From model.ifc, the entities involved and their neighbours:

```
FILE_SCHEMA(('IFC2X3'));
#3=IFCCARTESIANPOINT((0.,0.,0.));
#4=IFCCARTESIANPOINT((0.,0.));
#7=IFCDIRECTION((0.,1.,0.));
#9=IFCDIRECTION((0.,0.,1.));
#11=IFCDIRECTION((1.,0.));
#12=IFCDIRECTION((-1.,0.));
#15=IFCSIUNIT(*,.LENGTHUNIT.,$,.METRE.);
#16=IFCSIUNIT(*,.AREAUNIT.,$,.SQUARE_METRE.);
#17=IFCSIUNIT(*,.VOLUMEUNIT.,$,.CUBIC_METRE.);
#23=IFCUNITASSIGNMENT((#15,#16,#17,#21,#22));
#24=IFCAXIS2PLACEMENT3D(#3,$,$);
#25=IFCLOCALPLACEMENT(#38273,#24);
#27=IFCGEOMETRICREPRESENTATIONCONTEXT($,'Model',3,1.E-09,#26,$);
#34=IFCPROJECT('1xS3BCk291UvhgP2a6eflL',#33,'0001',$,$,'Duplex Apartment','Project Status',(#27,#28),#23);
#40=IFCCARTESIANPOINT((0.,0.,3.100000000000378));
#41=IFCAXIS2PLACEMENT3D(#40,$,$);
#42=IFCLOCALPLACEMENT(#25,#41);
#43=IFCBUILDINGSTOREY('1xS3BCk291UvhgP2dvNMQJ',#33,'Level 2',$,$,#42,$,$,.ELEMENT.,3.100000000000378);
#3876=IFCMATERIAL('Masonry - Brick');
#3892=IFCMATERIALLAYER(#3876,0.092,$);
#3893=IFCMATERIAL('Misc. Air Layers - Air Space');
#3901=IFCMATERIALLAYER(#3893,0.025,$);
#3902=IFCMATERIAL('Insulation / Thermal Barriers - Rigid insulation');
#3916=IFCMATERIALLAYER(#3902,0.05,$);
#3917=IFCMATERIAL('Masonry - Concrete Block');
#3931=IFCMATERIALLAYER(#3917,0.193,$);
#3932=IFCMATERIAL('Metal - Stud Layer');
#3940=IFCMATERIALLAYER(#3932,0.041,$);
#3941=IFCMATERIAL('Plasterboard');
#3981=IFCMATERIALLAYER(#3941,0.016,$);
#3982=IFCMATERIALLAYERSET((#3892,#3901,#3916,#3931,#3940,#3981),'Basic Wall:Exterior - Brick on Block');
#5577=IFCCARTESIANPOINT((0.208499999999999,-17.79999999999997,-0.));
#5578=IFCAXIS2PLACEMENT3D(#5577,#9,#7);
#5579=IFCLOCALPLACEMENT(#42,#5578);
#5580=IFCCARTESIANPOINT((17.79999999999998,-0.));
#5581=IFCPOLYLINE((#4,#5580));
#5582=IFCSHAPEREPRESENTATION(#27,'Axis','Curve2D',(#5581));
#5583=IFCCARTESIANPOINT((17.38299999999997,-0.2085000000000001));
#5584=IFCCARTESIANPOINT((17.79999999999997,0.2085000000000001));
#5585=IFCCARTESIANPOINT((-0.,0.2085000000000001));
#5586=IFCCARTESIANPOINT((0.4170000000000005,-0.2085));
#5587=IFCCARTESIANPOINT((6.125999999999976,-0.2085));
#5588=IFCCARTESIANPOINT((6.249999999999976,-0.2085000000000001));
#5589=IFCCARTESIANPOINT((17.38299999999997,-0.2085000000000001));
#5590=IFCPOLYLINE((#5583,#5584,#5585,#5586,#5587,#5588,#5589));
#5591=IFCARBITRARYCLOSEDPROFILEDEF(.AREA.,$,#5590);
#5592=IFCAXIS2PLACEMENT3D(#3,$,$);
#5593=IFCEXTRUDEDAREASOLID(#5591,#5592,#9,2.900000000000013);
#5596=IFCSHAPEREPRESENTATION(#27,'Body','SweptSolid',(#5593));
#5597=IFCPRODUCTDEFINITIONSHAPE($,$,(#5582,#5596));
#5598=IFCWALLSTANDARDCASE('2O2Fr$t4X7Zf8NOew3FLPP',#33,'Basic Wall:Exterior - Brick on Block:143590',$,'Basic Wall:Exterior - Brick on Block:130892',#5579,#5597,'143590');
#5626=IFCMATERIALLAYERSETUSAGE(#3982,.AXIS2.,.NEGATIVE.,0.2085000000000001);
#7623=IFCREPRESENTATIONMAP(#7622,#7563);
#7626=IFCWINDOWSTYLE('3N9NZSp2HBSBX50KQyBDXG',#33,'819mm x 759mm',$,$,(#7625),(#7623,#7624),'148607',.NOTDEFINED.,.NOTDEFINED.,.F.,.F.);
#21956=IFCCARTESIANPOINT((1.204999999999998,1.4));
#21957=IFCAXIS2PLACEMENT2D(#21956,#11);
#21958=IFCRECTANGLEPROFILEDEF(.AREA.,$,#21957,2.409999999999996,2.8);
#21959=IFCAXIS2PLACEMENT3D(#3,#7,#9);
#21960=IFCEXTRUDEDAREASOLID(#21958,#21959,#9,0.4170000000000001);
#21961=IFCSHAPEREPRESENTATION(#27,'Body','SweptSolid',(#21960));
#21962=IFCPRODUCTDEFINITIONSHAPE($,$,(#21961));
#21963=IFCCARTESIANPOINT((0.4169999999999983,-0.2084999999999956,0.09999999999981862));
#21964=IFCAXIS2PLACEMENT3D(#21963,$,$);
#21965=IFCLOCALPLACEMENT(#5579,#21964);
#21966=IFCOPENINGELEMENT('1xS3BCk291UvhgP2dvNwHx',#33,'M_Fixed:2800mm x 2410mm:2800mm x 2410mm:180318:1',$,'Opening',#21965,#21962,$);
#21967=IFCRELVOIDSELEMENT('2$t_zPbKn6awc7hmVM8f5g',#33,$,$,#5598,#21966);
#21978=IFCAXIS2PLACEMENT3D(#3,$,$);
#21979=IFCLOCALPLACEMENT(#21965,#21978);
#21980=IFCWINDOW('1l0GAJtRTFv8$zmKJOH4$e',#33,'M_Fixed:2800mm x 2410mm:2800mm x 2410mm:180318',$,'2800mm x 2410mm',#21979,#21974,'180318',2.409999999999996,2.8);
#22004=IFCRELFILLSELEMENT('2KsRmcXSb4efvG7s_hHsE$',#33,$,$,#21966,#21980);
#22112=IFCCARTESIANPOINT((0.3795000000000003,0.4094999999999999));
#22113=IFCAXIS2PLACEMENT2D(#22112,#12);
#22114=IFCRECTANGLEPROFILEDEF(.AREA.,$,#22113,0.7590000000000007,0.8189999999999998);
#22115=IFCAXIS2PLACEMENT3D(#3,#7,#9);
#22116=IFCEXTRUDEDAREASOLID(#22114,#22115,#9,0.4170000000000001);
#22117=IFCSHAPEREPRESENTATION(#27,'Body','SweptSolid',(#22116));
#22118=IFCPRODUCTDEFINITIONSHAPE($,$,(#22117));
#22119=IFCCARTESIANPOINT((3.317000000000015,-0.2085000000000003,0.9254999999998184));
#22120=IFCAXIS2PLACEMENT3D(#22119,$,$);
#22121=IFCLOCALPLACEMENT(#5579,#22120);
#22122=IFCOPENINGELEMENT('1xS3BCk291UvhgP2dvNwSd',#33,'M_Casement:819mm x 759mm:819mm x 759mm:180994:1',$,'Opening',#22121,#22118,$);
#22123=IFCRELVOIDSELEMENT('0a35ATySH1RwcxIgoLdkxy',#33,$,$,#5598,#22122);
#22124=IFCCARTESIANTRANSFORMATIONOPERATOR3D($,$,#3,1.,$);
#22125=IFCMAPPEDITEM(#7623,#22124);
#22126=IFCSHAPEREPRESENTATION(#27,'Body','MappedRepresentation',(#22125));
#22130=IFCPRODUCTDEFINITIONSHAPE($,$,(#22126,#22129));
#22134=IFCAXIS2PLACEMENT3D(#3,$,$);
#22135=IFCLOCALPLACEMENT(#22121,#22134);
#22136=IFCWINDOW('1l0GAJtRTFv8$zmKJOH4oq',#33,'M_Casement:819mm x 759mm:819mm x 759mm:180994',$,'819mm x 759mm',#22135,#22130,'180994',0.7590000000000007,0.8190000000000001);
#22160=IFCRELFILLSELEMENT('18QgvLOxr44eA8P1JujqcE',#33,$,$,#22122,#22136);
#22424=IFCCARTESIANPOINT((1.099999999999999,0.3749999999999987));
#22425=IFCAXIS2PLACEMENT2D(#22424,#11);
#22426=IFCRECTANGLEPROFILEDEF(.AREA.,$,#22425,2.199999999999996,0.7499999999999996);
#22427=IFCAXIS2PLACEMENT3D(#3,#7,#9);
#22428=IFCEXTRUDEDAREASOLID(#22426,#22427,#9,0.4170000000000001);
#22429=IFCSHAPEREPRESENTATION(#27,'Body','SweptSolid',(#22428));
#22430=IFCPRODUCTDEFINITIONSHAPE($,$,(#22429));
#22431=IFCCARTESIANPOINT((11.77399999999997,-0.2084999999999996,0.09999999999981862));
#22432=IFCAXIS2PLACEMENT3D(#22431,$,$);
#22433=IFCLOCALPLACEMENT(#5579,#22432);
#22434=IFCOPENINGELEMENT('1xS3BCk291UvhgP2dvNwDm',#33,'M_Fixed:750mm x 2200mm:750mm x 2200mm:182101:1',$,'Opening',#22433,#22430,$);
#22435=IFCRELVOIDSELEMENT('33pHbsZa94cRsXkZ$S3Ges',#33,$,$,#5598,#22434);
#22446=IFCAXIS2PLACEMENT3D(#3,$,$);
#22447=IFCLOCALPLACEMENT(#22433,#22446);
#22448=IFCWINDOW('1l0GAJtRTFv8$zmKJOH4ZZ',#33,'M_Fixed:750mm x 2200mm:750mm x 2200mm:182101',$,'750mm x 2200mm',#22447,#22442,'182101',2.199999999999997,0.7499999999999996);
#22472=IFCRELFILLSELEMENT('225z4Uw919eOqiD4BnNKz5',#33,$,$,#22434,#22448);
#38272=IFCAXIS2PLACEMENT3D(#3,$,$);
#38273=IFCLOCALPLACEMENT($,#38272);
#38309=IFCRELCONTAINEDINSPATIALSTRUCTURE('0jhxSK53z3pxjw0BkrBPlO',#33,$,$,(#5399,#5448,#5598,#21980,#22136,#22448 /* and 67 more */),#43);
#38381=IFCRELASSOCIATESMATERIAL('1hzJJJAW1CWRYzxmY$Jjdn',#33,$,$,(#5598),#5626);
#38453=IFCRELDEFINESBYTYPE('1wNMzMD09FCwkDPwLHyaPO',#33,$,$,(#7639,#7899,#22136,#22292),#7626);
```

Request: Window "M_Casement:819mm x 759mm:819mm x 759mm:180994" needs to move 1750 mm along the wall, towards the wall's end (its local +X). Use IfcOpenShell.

```python
import ifcopenshell
import ifcopenshell.api.geometry
import ifcopenshell.util.placement

model = ifcopenshell.open("model.ifc")

window = model.by_id(22136)
opening = window.FillsVoids[0].RelatingOpeningElement
wall = opening.VoidsElements[0].RelatingBuildingElement

wall_matrix = ifcopenshell.util.placement.get_local_placement(wall.ObjectPlacement)
shift = wall_matrix[:3, 0] * 1.75
before = ifcopenshell.util.placement.get_local_placement(window.ObjectPlacement)[:3, 3].copy()

# The window is placed relative to its opening, so it follows when the opening moves.
matrix = ifcopenshell.util.placement.get_local_placement(opening.ObjectPlacement)
matrix[:3, 3] += shift
ifcopenshell.api.geometry.edit_object_placement(
    model, product=opening, matrix=matrix, is_si=False, should_transform_children=True
)

after = ifcopenshell.util.placement.get_local_placement(window.ObjectPlacement)[:3, 3]
print("window moved by", (after - before).round(3) + 0.0)

model.write("model_edited.ifc")
```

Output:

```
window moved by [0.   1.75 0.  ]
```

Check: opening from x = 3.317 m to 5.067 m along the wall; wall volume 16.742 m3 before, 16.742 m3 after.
